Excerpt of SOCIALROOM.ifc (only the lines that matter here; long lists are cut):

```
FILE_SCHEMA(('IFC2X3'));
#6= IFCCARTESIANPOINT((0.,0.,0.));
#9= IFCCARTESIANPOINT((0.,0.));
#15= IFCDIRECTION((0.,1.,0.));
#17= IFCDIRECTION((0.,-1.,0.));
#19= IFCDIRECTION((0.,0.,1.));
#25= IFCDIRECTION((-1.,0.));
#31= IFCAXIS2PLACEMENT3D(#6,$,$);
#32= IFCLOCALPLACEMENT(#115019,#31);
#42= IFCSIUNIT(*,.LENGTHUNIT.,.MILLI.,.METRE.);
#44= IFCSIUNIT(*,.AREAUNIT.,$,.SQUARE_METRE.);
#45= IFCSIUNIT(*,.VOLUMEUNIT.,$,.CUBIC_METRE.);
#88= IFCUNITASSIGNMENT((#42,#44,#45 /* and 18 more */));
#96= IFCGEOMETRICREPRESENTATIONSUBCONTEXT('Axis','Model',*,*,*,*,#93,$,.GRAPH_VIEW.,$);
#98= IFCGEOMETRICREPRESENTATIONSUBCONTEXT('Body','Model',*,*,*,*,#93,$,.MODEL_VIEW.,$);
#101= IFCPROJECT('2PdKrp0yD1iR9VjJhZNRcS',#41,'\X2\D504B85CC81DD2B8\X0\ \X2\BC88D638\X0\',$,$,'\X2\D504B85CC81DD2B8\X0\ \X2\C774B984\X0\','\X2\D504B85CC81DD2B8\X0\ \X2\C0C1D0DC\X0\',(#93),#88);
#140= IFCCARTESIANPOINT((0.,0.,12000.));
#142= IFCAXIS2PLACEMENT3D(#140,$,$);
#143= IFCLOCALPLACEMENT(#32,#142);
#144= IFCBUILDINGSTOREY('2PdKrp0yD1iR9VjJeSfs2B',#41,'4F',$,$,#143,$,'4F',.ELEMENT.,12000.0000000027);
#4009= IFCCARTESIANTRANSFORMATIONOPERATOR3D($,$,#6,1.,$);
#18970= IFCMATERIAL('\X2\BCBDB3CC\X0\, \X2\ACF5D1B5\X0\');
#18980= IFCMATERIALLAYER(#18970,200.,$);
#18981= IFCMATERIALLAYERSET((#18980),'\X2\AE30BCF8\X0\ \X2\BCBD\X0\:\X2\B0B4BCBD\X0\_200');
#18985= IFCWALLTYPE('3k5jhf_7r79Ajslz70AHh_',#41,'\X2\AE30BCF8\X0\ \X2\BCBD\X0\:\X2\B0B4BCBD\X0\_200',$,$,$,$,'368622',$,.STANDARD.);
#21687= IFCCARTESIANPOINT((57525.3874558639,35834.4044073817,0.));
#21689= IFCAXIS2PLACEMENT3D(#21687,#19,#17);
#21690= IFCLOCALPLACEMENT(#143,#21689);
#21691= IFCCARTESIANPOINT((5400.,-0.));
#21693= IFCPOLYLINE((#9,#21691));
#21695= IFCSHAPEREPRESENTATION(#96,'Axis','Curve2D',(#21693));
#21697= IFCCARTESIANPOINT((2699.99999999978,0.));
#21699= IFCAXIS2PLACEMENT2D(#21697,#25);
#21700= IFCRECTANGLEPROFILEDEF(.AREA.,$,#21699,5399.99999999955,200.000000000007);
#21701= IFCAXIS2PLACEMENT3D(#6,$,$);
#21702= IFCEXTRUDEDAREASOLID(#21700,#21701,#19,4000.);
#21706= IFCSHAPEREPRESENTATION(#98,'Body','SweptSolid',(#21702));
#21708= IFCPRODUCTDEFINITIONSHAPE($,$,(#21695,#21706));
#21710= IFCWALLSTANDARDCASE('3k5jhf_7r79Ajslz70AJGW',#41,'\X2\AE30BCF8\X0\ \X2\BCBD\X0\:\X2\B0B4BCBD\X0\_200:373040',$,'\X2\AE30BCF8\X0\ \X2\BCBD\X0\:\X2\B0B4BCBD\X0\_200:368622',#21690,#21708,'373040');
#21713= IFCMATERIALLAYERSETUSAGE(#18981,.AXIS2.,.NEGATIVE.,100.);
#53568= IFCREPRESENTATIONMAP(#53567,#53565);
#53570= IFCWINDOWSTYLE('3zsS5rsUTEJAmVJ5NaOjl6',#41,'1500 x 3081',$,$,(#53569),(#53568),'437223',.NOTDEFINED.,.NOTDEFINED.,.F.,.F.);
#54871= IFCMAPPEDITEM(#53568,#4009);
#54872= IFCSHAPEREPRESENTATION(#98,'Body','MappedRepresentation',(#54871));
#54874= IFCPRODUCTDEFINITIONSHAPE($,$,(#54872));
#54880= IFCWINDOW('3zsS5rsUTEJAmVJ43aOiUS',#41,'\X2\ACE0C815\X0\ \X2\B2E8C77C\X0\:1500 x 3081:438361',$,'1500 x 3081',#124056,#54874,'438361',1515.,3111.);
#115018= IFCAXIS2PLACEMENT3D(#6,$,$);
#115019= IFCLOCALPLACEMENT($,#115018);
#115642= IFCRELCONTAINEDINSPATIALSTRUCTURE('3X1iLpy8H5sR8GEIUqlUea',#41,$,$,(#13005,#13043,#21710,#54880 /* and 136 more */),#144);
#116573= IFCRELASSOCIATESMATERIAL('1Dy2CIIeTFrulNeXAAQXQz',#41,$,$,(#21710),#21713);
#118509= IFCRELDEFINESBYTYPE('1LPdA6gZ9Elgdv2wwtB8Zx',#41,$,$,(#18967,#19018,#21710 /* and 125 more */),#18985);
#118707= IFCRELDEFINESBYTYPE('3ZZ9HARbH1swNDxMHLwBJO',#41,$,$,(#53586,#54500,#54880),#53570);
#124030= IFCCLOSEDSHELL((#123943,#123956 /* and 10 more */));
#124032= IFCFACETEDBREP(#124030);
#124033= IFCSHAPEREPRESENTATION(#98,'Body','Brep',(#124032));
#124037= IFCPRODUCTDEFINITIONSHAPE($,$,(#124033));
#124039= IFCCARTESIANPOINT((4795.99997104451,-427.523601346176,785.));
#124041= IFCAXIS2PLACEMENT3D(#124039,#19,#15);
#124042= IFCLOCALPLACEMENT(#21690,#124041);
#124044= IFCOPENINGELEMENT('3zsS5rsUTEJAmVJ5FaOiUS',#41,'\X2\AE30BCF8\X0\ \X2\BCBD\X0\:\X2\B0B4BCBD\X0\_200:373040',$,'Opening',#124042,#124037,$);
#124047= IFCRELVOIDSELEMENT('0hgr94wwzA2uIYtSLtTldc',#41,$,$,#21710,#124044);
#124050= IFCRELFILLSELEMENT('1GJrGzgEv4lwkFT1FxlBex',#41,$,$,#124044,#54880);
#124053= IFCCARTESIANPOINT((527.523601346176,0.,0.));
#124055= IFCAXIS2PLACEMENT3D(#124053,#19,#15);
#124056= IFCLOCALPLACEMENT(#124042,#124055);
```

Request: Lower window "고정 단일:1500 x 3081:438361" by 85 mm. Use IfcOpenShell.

```python
import numpy as np
import ifcopenshell
import ifcopenshell.api.geometry
import ifcopenshell.util.placement
import ifcopenshell.util.unit

model = ifcopenshell.open("SOCIALROOM.ifc")
unit_scale = ifcopenshell.util.unit.calculate_unit_scale(model)

window = model.by_guid("3zsS5rsUTEJAmVJ43aOiUS")
opening = window.FillsVoids[0].RelatingOpeningElement
dz = -0.085 / unit_scale

shift = np.array([0.0, 0.0, dz])
# The window is placed relative to its opening, so it follows when the opening moves.
matrix = ifcopenshell.util.placement.get_local_placement(opening.ObjectPlacement)
matrix[:3, 3] += shift
ifcopenshell.api.geometry.edit_object_placement(
    model, product=opening, matrix=matrix, is_si=False, should_transform_children=True
)

print(f"moved by {dz * unit_scale:+.3f} m")

model.write("SOCIALROOM_v2.ifc")
```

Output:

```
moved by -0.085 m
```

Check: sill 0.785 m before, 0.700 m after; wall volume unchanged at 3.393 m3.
